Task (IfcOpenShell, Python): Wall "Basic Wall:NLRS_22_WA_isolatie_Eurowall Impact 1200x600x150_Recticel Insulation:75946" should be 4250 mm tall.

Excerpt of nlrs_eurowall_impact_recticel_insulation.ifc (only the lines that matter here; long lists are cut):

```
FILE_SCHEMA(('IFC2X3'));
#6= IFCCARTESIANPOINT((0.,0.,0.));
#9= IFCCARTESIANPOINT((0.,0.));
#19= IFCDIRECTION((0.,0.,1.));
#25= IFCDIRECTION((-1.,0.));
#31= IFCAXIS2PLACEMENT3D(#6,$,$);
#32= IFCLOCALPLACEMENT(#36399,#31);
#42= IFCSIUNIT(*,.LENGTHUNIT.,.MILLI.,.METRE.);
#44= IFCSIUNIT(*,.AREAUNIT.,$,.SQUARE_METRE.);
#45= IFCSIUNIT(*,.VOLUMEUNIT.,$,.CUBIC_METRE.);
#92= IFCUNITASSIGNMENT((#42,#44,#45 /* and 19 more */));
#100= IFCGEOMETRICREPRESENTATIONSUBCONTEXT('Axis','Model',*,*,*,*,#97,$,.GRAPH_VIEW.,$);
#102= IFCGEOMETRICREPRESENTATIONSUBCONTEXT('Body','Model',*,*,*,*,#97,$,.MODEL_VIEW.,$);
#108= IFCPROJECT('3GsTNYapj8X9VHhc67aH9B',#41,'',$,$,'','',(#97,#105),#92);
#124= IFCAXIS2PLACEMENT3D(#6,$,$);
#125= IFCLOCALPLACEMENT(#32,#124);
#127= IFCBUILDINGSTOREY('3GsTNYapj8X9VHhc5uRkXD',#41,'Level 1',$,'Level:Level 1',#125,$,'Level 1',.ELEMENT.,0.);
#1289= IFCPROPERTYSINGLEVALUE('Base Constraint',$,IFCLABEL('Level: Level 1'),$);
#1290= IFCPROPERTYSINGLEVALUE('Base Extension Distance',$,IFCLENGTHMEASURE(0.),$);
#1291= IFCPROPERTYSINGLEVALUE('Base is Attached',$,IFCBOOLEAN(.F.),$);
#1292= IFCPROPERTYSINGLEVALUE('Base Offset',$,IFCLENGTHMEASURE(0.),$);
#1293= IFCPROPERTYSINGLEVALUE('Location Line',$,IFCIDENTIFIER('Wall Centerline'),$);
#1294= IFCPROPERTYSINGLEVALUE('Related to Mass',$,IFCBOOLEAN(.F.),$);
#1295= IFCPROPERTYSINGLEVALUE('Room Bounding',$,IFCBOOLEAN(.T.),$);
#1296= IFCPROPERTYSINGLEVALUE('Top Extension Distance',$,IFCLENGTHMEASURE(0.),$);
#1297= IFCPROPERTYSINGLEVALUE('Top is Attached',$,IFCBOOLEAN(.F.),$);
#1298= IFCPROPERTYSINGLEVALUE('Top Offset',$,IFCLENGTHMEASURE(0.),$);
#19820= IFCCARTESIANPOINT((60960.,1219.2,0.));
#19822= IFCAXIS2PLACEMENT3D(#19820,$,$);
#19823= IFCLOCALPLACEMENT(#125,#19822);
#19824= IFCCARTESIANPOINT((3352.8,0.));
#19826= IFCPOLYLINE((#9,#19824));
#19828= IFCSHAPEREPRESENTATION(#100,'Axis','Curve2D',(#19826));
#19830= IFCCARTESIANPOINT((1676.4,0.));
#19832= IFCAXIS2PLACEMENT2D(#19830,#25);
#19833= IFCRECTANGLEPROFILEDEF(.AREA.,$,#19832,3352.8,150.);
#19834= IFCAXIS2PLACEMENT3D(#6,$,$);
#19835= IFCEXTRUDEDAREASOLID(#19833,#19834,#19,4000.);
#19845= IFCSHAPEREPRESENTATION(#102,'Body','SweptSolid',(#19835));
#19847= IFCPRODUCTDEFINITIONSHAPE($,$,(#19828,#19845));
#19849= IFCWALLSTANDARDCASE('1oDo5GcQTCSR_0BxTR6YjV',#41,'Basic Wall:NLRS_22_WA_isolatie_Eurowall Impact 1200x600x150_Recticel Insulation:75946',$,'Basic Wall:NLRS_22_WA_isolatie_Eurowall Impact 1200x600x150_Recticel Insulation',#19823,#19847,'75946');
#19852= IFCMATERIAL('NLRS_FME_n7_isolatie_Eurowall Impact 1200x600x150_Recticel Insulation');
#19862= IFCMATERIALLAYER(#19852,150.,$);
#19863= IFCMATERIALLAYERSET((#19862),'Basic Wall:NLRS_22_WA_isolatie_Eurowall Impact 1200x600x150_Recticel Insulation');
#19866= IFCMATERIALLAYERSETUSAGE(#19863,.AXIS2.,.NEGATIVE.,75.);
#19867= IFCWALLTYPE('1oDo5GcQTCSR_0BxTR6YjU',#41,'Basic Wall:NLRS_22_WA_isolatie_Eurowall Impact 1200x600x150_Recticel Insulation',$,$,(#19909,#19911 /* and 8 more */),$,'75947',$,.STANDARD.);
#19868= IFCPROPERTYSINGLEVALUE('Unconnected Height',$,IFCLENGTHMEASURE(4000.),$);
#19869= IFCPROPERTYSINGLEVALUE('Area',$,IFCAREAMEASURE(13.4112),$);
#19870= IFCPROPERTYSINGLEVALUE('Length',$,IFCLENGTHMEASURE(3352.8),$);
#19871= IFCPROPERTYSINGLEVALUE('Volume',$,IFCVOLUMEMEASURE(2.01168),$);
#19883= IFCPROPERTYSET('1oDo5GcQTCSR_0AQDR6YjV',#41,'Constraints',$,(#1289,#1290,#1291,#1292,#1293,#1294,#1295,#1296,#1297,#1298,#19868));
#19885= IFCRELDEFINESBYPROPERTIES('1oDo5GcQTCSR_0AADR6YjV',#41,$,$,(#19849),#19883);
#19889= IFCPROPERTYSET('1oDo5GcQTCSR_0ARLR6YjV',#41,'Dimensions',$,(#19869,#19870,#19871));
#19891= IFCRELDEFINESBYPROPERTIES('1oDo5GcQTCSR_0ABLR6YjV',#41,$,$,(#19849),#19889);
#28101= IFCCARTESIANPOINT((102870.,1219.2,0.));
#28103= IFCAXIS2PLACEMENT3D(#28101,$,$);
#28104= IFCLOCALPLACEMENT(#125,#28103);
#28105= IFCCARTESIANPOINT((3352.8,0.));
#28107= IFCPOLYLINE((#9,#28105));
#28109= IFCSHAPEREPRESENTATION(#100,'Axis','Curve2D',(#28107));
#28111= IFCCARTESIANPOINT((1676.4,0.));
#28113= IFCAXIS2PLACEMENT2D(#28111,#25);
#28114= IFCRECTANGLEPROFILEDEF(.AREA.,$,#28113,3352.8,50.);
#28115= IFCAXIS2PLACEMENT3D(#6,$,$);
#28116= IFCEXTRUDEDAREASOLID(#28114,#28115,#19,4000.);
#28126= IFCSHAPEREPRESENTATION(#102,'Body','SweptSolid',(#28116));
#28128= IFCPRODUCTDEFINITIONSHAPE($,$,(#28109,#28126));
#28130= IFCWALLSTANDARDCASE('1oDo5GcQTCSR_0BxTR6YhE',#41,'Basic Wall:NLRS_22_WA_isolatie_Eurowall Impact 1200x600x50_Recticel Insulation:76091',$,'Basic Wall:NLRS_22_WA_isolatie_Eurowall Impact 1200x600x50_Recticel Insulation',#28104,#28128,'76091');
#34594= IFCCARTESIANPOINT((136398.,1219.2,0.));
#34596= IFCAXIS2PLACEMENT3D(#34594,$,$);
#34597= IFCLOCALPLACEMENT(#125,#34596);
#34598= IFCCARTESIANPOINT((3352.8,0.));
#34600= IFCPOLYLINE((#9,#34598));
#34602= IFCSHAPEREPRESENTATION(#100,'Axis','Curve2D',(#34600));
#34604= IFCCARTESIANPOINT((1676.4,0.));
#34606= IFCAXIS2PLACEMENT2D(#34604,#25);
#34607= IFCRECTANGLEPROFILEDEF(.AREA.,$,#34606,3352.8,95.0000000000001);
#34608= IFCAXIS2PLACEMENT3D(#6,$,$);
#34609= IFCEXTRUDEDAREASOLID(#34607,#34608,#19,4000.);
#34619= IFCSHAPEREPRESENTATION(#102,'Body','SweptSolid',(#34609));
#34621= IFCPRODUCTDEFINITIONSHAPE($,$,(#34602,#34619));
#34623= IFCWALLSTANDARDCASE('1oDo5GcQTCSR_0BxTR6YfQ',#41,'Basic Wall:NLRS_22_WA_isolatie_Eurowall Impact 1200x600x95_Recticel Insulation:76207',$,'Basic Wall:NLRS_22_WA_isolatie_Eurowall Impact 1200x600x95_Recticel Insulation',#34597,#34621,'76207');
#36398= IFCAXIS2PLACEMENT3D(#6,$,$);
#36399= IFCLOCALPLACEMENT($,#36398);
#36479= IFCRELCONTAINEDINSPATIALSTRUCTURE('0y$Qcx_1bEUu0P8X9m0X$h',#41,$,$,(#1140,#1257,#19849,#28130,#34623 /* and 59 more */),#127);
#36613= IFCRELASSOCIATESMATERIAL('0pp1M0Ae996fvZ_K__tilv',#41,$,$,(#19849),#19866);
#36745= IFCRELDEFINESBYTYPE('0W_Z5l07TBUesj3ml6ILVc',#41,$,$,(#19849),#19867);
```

```python
import ifcopenshell
import ifcopenshell.api.pset
import ifcopenshell.geom
import ifcopenshell.util.element
import ifcopenshell.util.representation
import ifcopenshell.util.shape
import ifcopenshell.util.unit

model = ifcopenshell.open("nlrs_eurowall_impact_recticel_insulation.ifc")
unit_scale = ifcopenshell.util.unit.calculate_unit_scale(model)
area_scale = ifcopenshell.util.unit.calculate_unit_scale(model, "AREAUNIT")
volume_scale = ifcopenshell.util.unit.calculate_unit_scale(model, "VOLUMEUNIT")
settings = ifcopenshell.geom.settings()


def volume(element):
    """Net volume in cubic metres, openings subtracted."""
    shape = ifcopenshell.geom.create_shape(settings, element)
    return ifcopenshell.util.shape.get_volume(shape.geometry)


wall = model.by_guid("1oDo5GcQTCSR_0BxTR6YjV")
before = volume(wall)

body = ifcopenshell.util.representation.get_representation(wall, "Model", "Body")
solid = body.Items[0]
old_height = solid.Depth
solid.Depth = 4.25 / unit_scale
after = volume(wall)
thickness = 0.15  # wall thickness in metres

# Update the stored height, areas and volumes.
pset = model.by_id(ifcopenshell.util.element.get_pset(wall, "Constraints", should_inherit=False)["id"])
ifcopenshell.api.pset.edit_pset(model, pset=pset, properties={
    "Unconnected Height": model.create_entity("IfcLengthMeasure", solid.Depth),
})
pset = model.by_id(ifcopenshell.util.element.get_pset(wall, "Dimensions", should_inherit=False)["id"])
ifcopenshell.api.pset.edit_pset(model, pset=pset, properties={
    "Area": model.create_entity("IfcAreaMeasure", after / thickness / area_scale),
    "Volume": model.create_entity("IfcVolumeMeasure", after / volume_scale),
})

print(f"height {old_height:g} -> {solid.Depth:g}, volume {before:.3f} -> {after:.3f} m3")

model.write("nlrs_eurowall_impact_recticel_insulation_rev.ifc")
```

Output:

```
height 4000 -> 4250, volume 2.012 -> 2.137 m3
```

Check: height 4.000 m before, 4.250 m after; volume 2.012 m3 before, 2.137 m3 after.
